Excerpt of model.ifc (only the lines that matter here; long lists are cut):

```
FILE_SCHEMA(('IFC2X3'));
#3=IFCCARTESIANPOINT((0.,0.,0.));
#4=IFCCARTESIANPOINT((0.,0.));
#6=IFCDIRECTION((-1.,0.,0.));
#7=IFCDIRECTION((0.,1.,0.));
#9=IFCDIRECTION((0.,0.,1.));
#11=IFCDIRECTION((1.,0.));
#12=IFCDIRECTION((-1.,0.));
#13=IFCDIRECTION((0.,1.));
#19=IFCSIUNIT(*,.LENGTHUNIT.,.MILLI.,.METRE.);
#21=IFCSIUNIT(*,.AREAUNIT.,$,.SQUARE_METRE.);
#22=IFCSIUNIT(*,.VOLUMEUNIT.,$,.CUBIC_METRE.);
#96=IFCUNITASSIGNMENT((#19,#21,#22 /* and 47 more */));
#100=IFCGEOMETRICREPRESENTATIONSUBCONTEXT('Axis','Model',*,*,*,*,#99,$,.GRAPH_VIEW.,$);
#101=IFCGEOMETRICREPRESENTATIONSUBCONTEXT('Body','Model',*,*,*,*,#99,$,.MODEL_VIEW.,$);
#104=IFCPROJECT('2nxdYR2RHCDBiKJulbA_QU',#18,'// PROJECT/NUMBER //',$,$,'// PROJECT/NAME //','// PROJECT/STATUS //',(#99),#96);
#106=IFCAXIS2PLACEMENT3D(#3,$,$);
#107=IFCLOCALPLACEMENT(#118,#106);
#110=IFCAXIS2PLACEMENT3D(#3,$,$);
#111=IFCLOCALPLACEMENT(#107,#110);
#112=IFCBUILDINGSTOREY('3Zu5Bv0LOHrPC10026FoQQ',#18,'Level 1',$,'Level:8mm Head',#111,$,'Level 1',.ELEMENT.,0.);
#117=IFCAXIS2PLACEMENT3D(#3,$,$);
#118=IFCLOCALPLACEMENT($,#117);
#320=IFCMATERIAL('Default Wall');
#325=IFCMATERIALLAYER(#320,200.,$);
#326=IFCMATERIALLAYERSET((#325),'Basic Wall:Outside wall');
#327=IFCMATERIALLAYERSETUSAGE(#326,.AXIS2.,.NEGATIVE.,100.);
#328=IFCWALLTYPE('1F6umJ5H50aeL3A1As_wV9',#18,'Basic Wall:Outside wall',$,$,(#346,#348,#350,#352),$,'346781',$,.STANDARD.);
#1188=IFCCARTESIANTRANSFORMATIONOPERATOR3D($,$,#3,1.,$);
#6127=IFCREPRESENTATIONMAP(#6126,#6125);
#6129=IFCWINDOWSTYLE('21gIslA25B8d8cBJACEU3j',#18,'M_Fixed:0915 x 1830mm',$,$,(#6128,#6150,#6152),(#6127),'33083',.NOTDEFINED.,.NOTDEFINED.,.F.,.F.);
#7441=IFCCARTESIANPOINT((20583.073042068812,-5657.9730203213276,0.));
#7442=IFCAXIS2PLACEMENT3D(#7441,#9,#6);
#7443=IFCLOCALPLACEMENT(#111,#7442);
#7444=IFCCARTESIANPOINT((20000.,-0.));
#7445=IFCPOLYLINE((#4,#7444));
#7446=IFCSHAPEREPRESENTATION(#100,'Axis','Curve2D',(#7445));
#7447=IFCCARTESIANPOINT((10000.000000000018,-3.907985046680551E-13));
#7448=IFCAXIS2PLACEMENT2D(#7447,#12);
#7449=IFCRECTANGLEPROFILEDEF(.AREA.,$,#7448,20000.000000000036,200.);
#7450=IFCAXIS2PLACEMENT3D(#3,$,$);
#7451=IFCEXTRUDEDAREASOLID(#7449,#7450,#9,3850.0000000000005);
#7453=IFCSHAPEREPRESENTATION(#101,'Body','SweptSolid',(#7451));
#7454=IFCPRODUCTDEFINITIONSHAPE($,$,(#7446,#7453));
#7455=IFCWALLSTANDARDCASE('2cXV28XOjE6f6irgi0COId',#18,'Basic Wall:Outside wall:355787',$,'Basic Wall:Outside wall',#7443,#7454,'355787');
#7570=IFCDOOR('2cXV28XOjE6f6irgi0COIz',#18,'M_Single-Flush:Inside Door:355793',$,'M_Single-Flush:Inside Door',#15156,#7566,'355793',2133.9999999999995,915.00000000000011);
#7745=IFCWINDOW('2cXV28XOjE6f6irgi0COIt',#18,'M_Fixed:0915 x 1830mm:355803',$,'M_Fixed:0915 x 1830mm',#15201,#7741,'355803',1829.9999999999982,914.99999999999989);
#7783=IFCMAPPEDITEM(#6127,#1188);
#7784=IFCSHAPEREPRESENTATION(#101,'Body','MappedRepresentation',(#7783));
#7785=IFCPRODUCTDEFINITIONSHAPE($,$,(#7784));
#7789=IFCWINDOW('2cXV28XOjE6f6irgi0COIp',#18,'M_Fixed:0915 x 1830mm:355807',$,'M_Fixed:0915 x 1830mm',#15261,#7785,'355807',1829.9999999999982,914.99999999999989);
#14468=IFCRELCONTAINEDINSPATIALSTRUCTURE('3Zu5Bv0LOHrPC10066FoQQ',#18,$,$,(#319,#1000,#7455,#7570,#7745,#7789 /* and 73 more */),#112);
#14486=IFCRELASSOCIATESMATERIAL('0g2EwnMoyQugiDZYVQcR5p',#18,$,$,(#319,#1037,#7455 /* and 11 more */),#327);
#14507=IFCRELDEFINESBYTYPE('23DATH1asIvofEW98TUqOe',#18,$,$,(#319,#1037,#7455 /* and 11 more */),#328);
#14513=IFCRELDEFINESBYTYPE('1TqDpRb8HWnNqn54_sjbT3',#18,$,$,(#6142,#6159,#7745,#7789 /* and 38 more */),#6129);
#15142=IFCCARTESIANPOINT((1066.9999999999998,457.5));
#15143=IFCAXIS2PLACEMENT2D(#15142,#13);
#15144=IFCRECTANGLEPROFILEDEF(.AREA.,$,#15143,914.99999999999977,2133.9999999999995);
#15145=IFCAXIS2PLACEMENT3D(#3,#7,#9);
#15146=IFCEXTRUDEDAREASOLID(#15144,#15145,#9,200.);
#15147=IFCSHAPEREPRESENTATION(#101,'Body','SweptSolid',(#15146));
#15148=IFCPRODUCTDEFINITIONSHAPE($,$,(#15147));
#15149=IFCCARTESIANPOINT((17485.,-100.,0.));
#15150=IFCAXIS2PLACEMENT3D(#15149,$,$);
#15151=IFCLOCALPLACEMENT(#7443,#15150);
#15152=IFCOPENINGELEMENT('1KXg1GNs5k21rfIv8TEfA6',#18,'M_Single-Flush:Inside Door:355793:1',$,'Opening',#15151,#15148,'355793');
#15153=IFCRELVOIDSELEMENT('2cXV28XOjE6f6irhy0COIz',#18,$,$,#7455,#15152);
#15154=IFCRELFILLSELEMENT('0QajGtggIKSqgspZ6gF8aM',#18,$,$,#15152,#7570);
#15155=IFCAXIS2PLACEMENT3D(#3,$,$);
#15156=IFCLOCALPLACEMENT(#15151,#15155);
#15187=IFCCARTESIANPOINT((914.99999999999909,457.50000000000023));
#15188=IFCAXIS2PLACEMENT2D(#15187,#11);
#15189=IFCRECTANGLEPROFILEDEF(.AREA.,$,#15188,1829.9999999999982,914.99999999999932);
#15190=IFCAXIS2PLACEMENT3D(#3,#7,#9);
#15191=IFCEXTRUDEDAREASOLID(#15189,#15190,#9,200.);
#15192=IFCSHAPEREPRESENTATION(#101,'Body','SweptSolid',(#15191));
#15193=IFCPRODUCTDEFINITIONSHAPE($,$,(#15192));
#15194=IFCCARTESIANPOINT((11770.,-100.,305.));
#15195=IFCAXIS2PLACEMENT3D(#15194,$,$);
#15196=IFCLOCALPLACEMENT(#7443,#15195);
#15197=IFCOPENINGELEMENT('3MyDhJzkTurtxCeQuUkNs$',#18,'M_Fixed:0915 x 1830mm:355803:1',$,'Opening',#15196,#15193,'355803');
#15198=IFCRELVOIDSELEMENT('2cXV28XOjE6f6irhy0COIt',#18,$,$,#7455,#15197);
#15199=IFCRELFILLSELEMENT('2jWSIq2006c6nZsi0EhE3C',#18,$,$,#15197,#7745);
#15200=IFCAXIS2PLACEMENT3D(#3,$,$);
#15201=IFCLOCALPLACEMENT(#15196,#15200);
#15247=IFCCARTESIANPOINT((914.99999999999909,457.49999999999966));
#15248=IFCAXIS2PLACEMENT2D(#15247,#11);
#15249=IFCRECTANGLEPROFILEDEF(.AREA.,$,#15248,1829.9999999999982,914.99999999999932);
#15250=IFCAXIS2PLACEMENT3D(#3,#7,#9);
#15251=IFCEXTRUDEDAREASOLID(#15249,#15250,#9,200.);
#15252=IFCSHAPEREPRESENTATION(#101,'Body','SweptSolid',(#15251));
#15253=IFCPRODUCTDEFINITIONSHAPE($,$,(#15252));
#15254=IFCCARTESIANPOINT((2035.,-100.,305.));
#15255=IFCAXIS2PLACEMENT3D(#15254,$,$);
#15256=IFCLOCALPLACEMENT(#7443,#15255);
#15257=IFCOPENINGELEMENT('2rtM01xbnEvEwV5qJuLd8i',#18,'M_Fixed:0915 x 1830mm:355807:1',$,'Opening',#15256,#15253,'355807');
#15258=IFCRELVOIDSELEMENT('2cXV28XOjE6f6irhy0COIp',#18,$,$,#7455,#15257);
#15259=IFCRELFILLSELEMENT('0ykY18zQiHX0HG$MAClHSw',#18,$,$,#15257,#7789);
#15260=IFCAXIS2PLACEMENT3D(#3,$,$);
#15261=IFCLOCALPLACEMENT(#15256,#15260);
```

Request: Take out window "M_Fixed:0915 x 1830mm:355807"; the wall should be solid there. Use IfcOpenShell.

```python
import ifcopenshell
import ifcopenshell.api.feature
import ifcopenshell.api.root
import ifcopenshell.geom
import ifcopenshell.util.shape

model = ifcopenshell.open("model.ifc")
settings = ifcopenshell.geom.settings()


def volume(element):
    """Net volume in cubic metres, openings subtracted."""
    shape = ifcopenshell.geom.create_shape(settings, element)
    return ifcopenshell.util.shape.get_volume(shape.geometry)


window = model.by_guid("2cXV28XOjE6f6irgi0COIp")
opening = window.FillsVoids[0].RelatingOpeningElement
wall = opening.VoidsElements[0].RelatingBuildingElement
before = volume(wall)

ifcopenshell.api.root.remove_product(model, product=window)
ifcopenshell.api.feature.remove_feature(model, feature=opening)

after = volume(wall)

print(f"wall volume {before:.3f} -> {after:.3f} m3")

model.write("model_updated.ifc")
```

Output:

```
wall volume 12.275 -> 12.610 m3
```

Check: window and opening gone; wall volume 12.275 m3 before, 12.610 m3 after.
